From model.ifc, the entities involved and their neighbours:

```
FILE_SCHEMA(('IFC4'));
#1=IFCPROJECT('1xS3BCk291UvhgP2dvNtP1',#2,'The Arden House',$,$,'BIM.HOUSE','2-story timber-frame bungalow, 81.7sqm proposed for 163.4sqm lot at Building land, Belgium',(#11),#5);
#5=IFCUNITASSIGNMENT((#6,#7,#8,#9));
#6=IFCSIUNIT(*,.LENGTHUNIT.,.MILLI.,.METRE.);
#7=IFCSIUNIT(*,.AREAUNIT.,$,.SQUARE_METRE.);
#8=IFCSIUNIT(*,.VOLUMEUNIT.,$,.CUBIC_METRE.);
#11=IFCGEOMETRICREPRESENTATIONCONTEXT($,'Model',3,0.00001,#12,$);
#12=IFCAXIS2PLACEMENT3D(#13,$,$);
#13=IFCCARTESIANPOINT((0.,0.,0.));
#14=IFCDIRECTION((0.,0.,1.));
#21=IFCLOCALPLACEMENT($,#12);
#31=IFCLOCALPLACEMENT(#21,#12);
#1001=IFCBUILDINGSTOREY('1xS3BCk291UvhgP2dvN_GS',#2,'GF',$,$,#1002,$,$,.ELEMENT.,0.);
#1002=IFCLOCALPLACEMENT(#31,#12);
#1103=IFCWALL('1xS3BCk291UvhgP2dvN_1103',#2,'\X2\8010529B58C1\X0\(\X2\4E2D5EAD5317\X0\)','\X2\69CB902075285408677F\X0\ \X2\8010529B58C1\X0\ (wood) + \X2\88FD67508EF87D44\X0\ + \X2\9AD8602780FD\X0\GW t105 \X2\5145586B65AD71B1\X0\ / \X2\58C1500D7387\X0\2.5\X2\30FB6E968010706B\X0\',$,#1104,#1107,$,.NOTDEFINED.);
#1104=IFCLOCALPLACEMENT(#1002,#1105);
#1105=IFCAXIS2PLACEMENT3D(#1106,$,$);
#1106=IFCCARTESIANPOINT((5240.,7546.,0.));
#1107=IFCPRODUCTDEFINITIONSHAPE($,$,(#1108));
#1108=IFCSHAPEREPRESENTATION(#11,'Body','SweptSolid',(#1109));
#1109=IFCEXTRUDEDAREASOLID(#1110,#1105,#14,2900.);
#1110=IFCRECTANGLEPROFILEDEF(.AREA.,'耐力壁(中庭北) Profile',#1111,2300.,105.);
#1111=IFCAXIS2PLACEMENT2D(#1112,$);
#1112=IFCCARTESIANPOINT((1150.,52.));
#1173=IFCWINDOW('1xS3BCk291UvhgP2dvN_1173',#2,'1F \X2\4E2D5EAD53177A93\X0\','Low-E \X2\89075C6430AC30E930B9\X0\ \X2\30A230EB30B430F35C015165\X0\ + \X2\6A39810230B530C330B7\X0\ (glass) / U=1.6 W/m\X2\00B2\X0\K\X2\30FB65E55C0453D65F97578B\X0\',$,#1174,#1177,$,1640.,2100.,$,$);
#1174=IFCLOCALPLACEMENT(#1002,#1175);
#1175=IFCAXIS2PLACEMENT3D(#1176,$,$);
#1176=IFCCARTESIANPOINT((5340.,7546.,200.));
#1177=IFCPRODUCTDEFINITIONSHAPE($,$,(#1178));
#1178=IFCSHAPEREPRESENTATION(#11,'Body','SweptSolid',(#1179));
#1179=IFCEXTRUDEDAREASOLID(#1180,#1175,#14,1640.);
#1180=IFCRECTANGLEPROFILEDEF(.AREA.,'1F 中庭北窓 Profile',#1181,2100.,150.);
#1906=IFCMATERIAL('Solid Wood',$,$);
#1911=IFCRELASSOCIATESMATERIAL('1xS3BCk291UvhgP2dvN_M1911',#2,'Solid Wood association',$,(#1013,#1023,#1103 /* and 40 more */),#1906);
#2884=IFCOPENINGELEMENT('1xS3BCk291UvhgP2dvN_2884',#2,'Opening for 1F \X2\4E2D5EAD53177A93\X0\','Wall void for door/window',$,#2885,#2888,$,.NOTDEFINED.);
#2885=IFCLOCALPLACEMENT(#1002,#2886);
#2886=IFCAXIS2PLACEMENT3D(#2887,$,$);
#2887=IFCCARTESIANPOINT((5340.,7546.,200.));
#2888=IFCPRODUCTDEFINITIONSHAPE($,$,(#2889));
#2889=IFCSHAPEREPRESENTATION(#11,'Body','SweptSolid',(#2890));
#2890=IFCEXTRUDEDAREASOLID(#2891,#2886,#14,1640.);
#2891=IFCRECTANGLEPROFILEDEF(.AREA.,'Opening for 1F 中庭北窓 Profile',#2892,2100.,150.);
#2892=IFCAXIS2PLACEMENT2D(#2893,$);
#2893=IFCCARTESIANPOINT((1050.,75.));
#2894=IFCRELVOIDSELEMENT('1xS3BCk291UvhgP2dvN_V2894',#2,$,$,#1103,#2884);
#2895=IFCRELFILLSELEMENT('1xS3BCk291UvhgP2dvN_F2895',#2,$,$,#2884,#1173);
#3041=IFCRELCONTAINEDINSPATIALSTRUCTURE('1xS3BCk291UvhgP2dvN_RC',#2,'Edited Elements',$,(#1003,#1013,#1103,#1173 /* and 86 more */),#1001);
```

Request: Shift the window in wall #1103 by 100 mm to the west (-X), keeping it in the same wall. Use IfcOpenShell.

```python
import ifcopenshell
import ifcopenshell.api.geometry
import ifcopenshell.util.placement
import ifcopenshell.util.unit

model = ifcopenshell.open("model.ifc")
unit_scale = ifcopenshell.util.unit.calculate_unit_scale(model)

window = model.by_id(1173)
opening = window.FillsVoids[0].RelatingOpeningElement
wall = opening.VoidsElements[0].RelatingBuildingElement

wall_matrix = ifcopenshell.util.placement.get_local_placement(wall.ObjectPlacement)
shift = wall_matrix[:3, 0] * -0.1 / unit_scale
before = ifcopenshell.util.placement.get_local_placement(window.ObjectPlacement)[:3, 3].copy()

# The window is not placed relative to its opening, so move both.
for product in (opening, window):
    matrix = ifcopenshell.util.placement.get_local_placement(product.ObjectPlacement)
    matrix[:3, 3] += shift
    ifcopenshell.api.geometry.edit_object_placement(model, product=product, matrix=matrix, is_si=False)

after = ifcopenshell.util.placement.get_local_placement(window.ObjectPlacement)[:3, 3]
print("window moved by", (after - before).round(3) + 0.0)

model.write("model_edited.ifc")
```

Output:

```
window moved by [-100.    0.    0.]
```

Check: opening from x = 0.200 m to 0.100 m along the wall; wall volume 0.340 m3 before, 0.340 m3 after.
